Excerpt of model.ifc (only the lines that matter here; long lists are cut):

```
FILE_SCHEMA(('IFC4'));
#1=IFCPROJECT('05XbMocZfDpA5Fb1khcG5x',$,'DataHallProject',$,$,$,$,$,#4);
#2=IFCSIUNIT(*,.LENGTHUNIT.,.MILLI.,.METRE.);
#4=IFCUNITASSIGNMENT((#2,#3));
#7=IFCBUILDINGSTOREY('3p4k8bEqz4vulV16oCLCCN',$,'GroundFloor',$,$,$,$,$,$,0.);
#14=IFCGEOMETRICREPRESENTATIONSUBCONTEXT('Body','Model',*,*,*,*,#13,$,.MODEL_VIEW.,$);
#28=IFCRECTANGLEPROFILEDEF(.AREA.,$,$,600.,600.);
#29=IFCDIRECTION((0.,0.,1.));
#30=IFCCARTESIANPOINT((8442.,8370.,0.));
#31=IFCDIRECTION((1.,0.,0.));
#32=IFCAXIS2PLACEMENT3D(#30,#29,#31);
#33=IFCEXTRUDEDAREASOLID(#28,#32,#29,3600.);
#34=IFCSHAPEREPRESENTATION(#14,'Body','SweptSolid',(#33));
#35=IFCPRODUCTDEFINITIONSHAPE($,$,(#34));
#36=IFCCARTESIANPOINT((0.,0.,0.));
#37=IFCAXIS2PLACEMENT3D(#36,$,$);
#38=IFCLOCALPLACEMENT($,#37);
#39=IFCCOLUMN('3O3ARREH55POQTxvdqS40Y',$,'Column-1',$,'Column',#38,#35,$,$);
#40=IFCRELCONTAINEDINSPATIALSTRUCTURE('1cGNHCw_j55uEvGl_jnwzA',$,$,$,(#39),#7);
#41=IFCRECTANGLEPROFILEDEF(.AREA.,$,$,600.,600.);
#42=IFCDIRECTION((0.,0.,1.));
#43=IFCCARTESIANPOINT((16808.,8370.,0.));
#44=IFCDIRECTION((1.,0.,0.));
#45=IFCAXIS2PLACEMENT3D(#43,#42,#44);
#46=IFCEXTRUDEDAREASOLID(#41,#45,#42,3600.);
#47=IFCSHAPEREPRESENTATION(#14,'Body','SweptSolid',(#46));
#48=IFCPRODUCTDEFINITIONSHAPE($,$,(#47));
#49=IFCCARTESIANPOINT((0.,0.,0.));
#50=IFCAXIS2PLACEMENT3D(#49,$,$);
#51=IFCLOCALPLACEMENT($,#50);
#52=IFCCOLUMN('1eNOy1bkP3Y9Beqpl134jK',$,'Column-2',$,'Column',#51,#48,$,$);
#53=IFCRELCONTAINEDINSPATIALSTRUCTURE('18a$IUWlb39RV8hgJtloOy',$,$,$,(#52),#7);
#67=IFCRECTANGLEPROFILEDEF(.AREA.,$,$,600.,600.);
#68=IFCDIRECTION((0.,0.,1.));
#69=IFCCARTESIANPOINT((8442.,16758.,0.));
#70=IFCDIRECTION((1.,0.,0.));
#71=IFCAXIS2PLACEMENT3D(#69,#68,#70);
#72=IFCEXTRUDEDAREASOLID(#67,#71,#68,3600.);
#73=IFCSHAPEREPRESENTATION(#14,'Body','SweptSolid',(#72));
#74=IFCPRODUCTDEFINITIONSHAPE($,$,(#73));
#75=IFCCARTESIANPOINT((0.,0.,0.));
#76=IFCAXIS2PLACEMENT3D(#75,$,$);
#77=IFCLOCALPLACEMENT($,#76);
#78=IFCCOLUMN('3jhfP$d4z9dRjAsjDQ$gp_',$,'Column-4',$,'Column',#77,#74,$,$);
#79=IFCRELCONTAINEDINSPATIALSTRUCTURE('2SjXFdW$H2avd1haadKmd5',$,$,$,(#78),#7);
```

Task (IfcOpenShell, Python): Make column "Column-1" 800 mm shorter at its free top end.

```python
import ifcopenshell
import ifcopenshell.util.representation

model = ifcopenshell.open("model.ifc")

member = model.by_guid("3O3ARREH55POQTxvdqS40Y")
change = -800.0

# The extrusion runs towards the end named, so only its depth changes.
body = ifcopenshell.util.representation.get_representation(member, "Model", "Body")
solid = body.Items[0]
old_length = solid.Depth
solid.Depth += change

print(f"length {old_length:g} -> {solid.Depth:g}")

model.write("model_v2.ifc")
```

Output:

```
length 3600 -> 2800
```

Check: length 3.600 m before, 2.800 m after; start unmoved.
